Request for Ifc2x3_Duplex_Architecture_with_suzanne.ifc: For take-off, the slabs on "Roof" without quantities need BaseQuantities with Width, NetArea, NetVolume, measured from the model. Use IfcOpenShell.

First a look at what the model holds.

```python
import ifcopenshell
import ifcopenshell.util.element
import ifcopenshell.util.unit

model = ifcopenshell.open("Ifc2x3_Duplex_Architecture_with_suzanne.ifc")
print(model.schema)
for unit_type in ("LENGTHUNIT", "AREAUNIT", "VOLUMEUNIT"):
    print(unit_type, ifcopenshell.util.unit.calculate_unit_scale(model, unit_type))
storey = next(s for s in model.by_type("IfcBuildingStorey") if s.Name == "Roof")
slabs = [e for e in ifcopenshell.util.element.get_decomposition(storey) if e.is_a("IfcSlab")]
for e in sorted(slabs, key=lambda e: e.id()):
    print(e.id(), e.is_a(), e.Name, list(ifcopenshell.util.element.get_psets(e, qtos_only=True)), sep=" | ")
```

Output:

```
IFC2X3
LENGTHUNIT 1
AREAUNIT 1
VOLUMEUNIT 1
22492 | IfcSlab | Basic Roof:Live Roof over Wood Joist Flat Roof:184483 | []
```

```python
import ifcopenshell
import ifcopenshell.api.pset
import ifcopenshell.geom
import ifcopenshell.util.element
import ifcopenshell.util.shape
import ifcopenshell.util.unit

model = ifcopenshell.open("Ifc2x3_Duplex_Architecture_with_suzanne.ifc")
unit_scale = ifcopenshell.util.unit.calculate_unit_scale(model)
area_scale = ifcopenshell.util.unit.calculate_unit_scale(model, "AREAUNIT")
volume_scale = ifcopenshell.util.unit.calculate_unit_scale(model, "VOLUMEUNIT")
settings = ifcopenshell.geom.settings()

storey = next(s for s in model.by_type("IfcBuildingStorey") if s.Name == "Roof")
slabs = [e for e in ifcopenshell.util.element.get_decomposition(storey) if e.is_a("IfcSlab")]

for e in sorted(slabs, key=lambda e: e.id()):
    if ifcopenshell.util.element.get_psets(e, qtos_only=True, should_inherit=False):
        continue
    # Geometry comes back in metres, in the element's own axes.
    shape = ifcopenshell.geom.create_shape(settings, e)
    values = {
        "Width": ifcopenshell.util.shape.get_z(shape.geometry) / unit_scale,
        "NetArea": ifcopenshell.util.shape.get_footprint_area(shape.geometry) / area_scale,
        "NetVolume": ifcopenshell.util.shape.get_volume(shape.geometry) / volume_scale,
    }
    qto = ifcopenshell.api.pset.add_qto(model, product=e, name="BaseQuantities")
    ifcopenshell.api.pset.edit_qto(model, qto=qto, properties=values)
    print(e.id(), {k: round(v, 3) for k, v in values.items()})

model.write("Ifc2x3_Duplex_Architecture_with_suzanne_edited.ifc")
```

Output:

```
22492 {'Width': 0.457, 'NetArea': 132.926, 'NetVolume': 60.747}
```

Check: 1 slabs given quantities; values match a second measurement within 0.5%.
